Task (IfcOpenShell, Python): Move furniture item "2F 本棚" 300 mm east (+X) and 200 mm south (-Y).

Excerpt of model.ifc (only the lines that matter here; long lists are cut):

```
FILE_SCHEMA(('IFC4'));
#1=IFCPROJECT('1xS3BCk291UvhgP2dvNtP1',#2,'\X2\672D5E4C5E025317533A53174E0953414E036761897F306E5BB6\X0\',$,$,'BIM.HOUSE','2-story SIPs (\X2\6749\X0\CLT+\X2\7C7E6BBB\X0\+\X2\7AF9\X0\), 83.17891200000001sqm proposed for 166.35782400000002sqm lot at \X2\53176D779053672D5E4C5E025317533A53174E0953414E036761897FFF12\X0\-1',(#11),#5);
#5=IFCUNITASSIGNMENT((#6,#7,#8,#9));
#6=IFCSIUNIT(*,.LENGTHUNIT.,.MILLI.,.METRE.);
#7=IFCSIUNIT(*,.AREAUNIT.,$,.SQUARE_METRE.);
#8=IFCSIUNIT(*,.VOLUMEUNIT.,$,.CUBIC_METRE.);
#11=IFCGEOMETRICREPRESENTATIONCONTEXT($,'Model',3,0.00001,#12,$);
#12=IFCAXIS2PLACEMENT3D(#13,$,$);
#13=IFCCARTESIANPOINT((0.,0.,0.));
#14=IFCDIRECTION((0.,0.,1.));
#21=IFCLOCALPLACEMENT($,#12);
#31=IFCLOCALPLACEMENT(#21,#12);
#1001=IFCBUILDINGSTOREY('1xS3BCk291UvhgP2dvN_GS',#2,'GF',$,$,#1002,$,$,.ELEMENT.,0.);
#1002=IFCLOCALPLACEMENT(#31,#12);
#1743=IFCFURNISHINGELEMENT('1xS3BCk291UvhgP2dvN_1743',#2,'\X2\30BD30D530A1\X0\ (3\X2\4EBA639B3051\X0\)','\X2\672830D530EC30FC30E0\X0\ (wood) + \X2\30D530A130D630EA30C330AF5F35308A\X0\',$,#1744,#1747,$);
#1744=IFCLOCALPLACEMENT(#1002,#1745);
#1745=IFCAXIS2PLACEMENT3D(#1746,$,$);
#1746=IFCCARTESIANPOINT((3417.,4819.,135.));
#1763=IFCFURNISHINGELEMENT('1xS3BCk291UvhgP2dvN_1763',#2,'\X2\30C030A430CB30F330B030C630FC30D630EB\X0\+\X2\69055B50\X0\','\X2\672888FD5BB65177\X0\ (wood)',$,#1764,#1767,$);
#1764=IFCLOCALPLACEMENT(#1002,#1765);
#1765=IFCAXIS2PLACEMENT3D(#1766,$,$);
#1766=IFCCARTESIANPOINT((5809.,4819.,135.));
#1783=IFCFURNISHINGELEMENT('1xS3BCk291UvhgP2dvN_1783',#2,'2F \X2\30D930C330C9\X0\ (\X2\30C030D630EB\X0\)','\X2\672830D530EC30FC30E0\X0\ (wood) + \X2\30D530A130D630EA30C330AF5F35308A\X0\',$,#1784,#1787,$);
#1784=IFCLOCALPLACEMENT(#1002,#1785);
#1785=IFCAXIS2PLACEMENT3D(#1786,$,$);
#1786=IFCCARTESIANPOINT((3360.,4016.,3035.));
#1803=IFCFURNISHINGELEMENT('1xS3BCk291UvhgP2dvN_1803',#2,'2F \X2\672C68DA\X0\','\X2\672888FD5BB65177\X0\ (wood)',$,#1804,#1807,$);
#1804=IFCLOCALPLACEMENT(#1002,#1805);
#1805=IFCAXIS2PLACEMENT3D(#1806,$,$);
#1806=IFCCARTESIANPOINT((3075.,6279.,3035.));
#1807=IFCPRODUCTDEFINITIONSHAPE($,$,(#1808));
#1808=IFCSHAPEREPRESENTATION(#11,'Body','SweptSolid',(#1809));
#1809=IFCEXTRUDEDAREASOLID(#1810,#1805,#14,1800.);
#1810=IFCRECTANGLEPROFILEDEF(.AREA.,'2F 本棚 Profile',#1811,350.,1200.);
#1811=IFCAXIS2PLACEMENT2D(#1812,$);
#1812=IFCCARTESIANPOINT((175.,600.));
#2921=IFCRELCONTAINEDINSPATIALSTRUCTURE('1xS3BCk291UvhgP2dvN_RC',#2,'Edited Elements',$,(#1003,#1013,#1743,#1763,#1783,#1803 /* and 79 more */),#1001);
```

```python
import ifcopenshell
import ifcopenshell.api.geometry
import ifcopenshell.util.placement

model = ifcopenshell.open("model.ifc")

item = model.by_guid("1xS3BCk291UvhgP2dvN_1803")
matrix = ifcopenshell.util.placement.get_local_placement(item.ObjectPlacement)
matrix[0, 3] += 300.0
matrix[1, 3] -= 200.0
ifcopenshell.api.geometry.edit_object_placement(model, product=item, matrix=matrix, is_si=False)

print(ifcopenshell.util.placement.get_local_placement(item.ObjectPlacement).round(3) + 0.0)

model.write("model_edited.ifc")
```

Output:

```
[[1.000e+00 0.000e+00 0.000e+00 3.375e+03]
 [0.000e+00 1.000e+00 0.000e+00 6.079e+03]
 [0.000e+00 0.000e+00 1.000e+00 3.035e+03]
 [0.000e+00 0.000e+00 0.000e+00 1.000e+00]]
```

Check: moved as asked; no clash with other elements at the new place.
